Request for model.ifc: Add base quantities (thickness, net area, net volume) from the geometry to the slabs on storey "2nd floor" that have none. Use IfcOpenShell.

First a look at what the model holds.

```python
import ifcopenshell
import ifcopenshell.util.element
import ifcopenshell.util.unit

model = ifcopenshell.open("model.ifc")
print(model.schema)
for unit_type in ("LENGTHUNIT", "AREAUNIT", "VOLUMEUNIT"):
    print(unit_type, ifcopenshell.util.unit.calculate_unit_scale(model, unit_type))
storey = next(s for s in model.by_type("IfcBuildingStorey") if s.Name == "2nd floor")
slabs = [e for e in ifcopenshell.util.element.get_decomposition(storey) if e.is_a("IfcSlab")]
for e in sorted(slabs, key=lambda e: e.id()):
    print(e.id(), e.is_a(), e.Name, list(ifcopenshell.util.element.get_psets(e, qtos_only=True)), sep=" | ")
```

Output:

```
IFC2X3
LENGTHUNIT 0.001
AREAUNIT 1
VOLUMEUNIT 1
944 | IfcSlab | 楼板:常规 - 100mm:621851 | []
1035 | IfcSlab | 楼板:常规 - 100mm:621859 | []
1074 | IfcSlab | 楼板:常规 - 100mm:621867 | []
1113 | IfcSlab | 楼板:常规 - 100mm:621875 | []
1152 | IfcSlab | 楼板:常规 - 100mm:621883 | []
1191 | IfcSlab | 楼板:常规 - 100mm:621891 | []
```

```python
import ifcopenshell
import ifcopenshell.api.pset
import ifcopenshell.geom
import ifcopenshell.util.element
import ifcopenshell.util.shape
import ifcopenshell.util.unit

model = ifcopenshell.open("model.ifc")
unit_scale = ifcopenshell.util.unit.calculate_unit_scale(model)
area_scale = ifcopenshell.util.unit.calculate_unit_scale(model, "AREAUNIT")
volume_scale = ifcopenshell.util.unit.calculate_unit_scale(model, "VOLUMEUNIT")
settings = ifcopenshell.geom.settings()

storey = next(s for s in model.by_type("IfcBuildingStorey") if s.Name == "2nd floor")
slabs = [e for e in ifcopenshell.util.element.get_decomposition(storey) if e.is_a("IfcSlab")]

for e in sorted(slabs, key=lambda e: e.id()):
    if ifcopenshell.util.element.get_psets(e, qtos_only=True, should_inherit=False):
        continue
    # Geometry comes back in metres, in the element's own axes.
    shape = ifcopenshell.geom.create_shape(settings, e)
    values = {
        "Width": ifcopenshell.util.shape.get_z(shape.geometry) / unit_scale,
        "NetArea": ifcopenshell.util.shape.get_footprint_area(shape.geometry) / area_scale,
        "NetVolume": ifcopenshell.util.shape.get_volume(shape.geometry) / volume_scale,
    }
    qto = ifcopenshell.api.pset.add_qto(model, product=e, name="BaseQuantities")
    ifcopenshell.api.pset.edit_qto(model, qto=qto, properties=values)
    print(e.id(), {k: round(v, 3) for k, v in values.items()})

model.write("model_edited.ifc")
```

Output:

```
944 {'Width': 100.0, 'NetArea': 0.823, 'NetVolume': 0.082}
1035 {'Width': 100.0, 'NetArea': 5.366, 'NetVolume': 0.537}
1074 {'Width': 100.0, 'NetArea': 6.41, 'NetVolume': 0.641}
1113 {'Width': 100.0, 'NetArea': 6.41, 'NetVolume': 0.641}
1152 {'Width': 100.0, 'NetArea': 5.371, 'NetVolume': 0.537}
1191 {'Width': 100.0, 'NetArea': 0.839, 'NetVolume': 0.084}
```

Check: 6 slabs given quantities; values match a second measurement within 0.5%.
